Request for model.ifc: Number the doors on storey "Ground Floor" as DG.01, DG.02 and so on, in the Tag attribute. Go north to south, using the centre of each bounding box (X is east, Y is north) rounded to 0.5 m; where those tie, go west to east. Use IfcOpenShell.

First a look at what the model holds.

```python
import ifcopenshell
import ifcopenshell.util.element
import ifcopenshell.util.placement

model = ifcopenshell.open("model.ifc")
print(model.schema)
storey = next(s for s in model.by_type("IfcBuildingStorey") if s.Name == "Ground Floor")
doors = [e for e in ifcopenshell.util.element.get_decomposition(storey) if e.is_a("IfcDoor")]
for e in sorted(doors, key=lambda e: e.id()):
    origin = ifcopenshell.util.placement.get_local_placement(e.ObjectPlacement)[:3, 3]
    print(e.id(), e.Tag, e.Name, origin.round(2) + 0.0, sep=" | ")
```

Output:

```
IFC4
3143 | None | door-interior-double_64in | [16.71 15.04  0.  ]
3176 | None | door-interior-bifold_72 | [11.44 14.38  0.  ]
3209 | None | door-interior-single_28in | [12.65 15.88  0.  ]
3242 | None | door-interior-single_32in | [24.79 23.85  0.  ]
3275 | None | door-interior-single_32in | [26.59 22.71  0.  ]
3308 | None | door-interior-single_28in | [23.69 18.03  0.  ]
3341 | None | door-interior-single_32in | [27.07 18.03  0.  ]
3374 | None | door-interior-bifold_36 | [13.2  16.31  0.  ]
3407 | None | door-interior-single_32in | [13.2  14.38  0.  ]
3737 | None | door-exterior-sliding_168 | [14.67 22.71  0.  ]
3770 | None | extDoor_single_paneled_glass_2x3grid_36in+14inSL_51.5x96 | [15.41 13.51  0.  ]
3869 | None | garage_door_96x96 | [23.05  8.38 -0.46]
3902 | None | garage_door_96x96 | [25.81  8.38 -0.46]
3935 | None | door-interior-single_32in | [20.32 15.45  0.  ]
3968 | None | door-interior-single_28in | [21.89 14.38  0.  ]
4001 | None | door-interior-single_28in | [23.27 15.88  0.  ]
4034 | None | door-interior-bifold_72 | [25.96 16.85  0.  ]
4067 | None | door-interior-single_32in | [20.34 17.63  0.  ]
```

```python
import ifcopenshell
import ifcopenshell.geom
import ifcopenshell.util.element
import ifcopenshell.util.shape

model = ifcopenshell.open("model.ifc")
settings = ifcopenshell.geom.settings()
settings.set("use-world-coords", True)


def centre(element):
    shape = ifcopenshell.geom.create_shape(settings, element)
    return ifcopenshell.util.shape.get_bbox_centroid(shape.geometry)


storey = next(s for s in model.by_type("IfcBuildingStorey") if s.Name == "Ground Floor")
doors = [e for e in ifcopenshell.util.element.get_decomposition(storey) if e.is_a("IfcDoor")]

# Insertion points can sit at a corner or the storey origin, so sort by the geometry (in metres).
centres = {e: centre(e) for e in doors}
doors.sort(key=lambda e: (-round(centres[e][1] / 0.5), centres[e][0]))

for i, e in enumerate(doors, start=1):
    number = f"DG.{i:02d}"
    e.Tag = number
    print(e.id(), number)

model.write("model_updated.ifc")
```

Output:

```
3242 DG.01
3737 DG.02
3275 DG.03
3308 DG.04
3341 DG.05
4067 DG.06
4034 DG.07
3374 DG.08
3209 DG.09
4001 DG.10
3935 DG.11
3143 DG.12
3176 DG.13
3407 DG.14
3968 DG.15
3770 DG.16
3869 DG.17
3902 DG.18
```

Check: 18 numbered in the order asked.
